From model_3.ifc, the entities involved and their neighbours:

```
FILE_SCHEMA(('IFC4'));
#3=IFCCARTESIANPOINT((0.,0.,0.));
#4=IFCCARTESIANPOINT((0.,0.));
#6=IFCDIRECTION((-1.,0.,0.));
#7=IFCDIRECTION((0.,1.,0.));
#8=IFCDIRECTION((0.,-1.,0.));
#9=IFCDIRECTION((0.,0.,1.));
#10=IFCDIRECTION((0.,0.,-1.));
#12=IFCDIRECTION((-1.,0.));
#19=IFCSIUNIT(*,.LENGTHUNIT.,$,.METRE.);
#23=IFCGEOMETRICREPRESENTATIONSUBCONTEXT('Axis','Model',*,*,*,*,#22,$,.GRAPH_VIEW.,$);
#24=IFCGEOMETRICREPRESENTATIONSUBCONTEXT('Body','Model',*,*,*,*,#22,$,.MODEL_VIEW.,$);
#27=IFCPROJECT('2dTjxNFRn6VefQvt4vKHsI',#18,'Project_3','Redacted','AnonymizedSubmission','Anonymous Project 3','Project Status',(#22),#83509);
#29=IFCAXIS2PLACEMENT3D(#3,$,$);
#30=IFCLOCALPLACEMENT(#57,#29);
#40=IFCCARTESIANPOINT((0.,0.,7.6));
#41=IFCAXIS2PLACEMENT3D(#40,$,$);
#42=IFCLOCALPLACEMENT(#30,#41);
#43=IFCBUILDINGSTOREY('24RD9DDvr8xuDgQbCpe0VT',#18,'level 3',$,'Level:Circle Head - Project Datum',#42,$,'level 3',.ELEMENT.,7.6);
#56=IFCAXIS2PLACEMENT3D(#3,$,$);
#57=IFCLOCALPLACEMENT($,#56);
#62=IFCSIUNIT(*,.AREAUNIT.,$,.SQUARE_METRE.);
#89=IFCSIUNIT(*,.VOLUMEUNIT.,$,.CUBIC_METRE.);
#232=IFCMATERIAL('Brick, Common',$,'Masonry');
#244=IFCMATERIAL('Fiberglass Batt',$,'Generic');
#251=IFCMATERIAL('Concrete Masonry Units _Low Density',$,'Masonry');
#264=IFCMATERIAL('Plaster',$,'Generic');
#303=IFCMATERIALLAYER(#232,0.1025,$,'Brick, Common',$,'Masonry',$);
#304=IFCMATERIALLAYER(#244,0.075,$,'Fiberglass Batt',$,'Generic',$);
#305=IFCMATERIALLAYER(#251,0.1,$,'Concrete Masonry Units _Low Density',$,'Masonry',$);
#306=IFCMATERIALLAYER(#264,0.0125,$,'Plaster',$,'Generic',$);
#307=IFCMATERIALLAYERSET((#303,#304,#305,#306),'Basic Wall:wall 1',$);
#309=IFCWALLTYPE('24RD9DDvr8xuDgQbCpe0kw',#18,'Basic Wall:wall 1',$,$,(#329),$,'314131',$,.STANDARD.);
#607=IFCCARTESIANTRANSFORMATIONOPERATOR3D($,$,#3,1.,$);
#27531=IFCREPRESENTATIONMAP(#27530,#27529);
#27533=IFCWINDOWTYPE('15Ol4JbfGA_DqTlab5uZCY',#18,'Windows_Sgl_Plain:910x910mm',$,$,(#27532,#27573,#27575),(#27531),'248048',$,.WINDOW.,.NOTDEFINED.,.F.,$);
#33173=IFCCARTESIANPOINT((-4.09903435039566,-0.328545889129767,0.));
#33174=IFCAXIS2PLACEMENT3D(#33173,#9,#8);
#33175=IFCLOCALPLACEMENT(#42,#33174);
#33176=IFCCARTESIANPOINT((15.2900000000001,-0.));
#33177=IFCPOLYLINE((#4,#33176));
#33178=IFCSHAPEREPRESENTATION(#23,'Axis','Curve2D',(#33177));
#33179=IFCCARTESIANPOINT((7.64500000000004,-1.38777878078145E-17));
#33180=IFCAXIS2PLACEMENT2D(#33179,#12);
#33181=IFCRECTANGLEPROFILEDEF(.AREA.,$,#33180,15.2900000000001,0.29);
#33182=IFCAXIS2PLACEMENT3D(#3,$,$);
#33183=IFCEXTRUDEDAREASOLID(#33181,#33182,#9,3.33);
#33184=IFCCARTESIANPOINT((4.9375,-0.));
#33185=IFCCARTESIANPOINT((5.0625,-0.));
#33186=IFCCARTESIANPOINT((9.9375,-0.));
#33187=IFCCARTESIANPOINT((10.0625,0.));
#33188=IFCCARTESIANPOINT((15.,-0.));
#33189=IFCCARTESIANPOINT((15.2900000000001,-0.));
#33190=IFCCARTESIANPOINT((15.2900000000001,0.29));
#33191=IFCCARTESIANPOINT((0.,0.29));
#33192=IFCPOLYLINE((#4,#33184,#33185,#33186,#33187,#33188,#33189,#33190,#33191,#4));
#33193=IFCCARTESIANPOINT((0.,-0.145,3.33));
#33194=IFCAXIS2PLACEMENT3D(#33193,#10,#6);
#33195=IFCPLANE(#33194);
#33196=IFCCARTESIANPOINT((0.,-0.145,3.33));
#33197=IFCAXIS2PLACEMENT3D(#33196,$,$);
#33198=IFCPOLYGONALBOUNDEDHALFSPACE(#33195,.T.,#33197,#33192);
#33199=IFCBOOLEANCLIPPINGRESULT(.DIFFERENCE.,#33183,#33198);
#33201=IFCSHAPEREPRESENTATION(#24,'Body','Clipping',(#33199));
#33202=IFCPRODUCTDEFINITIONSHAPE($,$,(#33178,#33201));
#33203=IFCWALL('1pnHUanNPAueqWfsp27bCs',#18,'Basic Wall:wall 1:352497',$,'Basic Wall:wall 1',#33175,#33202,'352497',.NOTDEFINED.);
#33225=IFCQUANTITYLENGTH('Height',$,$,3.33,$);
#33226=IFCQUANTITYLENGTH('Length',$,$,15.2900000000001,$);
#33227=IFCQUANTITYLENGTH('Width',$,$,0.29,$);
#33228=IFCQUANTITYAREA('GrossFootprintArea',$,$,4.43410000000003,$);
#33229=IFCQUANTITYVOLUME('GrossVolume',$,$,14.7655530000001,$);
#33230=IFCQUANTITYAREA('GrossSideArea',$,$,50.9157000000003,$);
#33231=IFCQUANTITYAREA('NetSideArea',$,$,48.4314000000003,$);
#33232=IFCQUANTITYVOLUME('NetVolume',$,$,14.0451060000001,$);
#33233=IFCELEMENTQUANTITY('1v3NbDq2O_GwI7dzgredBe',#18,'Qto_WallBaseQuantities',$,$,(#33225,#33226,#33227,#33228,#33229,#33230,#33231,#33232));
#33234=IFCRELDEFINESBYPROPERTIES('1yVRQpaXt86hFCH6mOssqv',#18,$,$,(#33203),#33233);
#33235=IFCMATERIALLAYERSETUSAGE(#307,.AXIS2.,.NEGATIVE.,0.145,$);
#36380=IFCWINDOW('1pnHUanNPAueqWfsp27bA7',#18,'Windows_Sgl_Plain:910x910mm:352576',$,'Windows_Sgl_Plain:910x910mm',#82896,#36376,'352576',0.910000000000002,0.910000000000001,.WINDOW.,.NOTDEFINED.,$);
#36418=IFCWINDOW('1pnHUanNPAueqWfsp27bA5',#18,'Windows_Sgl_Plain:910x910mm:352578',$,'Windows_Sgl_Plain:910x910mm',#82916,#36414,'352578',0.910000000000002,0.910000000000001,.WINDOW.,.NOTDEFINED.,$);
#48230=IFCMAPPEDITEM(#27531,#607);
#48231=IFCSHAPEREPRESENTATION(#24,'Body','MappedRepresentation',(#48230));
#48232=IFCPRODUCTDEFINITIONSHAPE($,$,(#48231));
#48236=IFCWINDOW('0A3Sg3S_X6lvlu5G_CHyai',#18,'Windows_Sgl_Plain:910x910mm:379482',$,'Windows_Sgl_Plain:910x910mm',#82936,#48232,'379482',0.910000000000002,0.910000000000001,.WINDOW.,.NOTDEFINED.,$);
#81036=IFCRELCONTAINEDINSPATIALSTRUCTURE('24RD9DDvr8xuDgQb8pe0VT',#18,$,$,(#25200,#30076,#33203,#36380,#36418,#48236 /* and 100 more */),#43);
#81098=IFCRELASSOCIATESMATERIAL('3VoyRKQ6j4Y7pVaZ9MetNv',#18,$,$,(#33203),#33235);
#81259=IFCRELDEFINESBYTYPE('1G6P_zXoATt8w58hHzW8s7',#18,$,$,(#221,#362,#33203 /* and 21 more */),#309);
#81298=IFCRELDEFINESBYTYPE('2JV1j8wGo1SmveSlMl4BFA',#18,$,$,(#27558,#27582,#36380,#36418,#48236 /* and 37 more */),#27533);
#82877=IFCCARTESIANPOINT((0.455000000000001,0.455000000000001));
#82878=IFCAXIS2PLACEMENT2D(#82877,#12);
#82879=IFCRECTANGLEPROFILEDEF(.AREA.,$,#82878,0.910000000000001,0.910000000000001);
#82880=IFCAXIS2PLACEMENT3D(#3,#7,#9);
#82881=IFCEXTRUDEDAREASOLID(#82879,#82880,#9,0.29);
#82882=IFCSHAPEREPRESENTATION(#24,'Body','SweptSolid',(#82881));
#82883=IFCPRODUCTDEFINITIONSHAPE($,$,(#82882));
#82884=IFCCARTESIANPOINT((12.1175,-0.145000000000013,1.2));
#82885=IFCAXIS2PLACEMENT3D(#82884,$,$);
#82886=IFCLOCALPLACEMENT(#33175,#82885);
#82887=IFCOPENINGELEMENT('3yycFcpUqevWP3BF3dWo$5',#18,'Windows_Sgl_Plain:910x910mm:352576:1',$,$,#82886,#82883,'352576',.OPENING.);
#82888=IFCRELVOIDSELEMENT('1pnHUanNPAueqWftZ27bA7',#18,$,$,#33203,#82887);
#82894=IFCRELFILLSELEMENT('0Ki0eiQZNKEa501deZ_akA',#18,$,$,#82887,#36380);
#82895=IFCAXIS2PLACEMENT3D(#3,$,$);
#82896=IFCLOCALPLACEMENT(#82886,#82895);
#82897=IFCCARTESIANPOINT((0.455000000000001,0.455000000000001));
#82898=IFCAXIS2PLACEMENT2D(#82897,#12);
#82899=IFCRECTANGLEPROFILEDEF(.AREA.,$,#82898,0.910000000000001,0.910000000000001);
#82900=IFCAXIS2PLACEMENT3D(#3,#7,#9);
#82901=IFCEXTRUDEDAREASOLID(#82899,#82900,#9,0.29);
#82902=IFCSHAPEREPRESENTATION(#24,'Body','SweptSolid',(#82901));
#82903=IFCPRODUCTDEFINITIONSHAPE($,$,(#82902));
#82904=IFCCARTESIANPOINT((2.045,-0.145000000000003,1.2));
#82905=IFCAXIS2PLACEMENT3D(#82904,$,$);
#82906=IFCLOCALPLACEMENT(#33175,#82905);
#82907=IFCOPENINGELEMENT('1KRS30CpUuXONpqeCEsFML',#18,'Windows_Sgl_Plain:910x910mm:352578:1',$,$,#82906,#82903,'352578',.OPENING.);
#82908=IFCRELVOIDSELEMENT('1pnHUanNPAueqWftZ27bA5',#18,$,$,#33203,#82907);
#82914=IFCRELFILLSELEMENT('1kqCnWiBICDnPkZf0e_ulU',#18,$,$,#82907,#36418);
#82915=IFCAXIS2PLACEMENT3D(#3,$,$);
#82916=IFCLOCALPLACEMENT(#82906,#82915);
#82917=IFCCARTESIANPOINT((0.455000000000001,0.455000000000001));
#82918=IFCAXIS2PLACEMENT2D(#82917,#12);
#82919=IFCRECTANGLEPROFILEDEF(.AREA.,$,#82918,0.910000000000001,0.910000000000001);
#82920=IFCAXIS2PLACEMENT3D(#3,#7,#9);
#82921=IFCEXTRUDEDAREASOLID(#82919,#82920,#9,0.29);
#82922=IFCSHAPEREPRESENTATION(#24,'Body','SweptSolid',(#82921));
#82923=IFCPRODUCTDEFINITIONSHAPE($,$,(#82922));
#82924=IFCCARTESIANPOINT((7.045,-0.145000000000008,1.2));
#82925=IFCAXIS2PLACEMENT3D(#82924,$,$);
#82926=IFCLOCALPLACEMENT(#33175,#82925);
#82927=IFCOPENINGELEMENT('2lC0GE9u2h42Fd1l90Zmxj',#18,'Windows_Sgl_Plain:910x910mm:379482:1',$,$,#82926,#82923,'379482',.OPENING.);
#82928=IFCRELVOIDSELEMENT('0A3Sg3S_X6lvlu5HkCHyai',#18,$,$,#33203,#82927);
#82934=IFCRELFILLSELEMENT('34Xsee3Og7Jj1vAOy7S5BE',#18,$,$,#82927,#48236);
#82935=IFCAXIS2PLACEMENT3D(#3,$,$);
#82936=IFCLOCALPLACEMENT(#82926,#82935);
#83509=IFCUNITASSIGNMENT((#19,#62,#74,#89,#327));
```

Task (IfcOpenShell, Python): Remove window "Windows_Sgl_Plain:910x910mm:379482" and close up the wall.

```python
import ifcopenshell
import ifcopenshell.api.feature
import ifcopenshell.api.pset
import ifcopenshell.api.root
import ifcopenshell.geom
import ifcopenshell.util.element
import ifcopenshell.util.shape
import ifcopenshell.util.unit

model = ifcopenshell.open("model_3.ifc")
area_scale = ifcopenshell.util.unit.calculate_unit_scale(model, "AREAUNIT")
volume_scale = ifcopenshell.util.unit.calculate_unit_scale(model, "VOLUMEUNIT")
settings = ifcopenshell.geom.settings()


def volume(element):
    """Net volume in cubic metres, openings subtracted."""
    shape = ifcopenshell.geom.create_shape(settings, element)
    return ifcopenshell.util.shape.get_volume(shape.geometry)


window = model.by_guid("0A3Sg3S_X6lvlu5G_CHyai")
opening = window.FillsVoids[0].RelatingOpeningElement
wall = opening.VoidsElements[0].RelatingBuildingElement
before = volume(wall)

ifcopenshell.api.root.remove_product(model, product=window)
ifcopenshell.api.feature.remove_feature(model, feature=opening)

after = volume(wall)
thickness = 0.29  # wall thickness in metres

# Update the wall's stored quantities.
qto = model.by_id(ifcopenshell.util.element.get_pset(wall, "Qto_WallBaseQuantities", should_inherit=False)["id"])
ifcopenshell.api.pset.edit_qto(model, qto=qto, properties={
    "NetSideArea": after / thickness / area_scale,
    "NetVolume": after / volume_scale,
})

print(f"wall volume {before:.3f} -> {after:.3f} m3")

model.write("model_3-out.ifc")
```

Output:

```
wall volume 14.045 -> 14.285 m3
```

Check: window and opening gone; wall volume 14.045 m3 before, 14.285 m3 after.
